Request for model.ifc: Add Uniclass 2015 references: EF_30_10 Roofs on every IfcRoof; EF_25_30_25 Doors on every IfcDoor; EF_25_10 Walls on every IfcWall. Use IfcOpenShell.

First a look at what the model holds.

```python
import ifcopenshell

model = ifcopenshell.open("model.ifc")
print(model.schema)
print("classifications:", [c.Name for c in model.by_type("IfcClassification")])
for ifc_class in ("IfcDoor", "IfcRoof", "IfcStair", "IfcWall", "IfcWindow"):
    print(ifc_class, len(model.by_type(ifc_class)))
```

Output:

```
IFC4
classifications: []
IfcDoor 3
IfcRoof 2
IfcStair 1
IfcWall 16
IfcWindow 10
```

```python
import ifcopenshell
import ifcopenshell.api.classification

model = ifcopenshell.open("model.ifc")

system = ifcopenshell.api.classification.add_classification(model, classification="Uniclass 2015")

codes = {
    "IfcRoof": ("EF_30_10", "Roofs"),
    "IfcDoor": ("EF_25_30_25", "Doors"),
    "IfcWall": ("EF_25_10", "Walls"),
}
for ifc_class, (code, name) in codes.items():
    products = model.by_type(ifc_class)
    ifcopenshell.api.classification.add_reference(
        model, products=products, classification=system, identification=code, name=name
    )
    print(code, len(products))

model.write("model_v2.ifc")
```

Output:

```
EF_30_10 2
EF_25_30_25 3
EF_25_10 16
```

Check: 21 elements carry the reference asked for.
